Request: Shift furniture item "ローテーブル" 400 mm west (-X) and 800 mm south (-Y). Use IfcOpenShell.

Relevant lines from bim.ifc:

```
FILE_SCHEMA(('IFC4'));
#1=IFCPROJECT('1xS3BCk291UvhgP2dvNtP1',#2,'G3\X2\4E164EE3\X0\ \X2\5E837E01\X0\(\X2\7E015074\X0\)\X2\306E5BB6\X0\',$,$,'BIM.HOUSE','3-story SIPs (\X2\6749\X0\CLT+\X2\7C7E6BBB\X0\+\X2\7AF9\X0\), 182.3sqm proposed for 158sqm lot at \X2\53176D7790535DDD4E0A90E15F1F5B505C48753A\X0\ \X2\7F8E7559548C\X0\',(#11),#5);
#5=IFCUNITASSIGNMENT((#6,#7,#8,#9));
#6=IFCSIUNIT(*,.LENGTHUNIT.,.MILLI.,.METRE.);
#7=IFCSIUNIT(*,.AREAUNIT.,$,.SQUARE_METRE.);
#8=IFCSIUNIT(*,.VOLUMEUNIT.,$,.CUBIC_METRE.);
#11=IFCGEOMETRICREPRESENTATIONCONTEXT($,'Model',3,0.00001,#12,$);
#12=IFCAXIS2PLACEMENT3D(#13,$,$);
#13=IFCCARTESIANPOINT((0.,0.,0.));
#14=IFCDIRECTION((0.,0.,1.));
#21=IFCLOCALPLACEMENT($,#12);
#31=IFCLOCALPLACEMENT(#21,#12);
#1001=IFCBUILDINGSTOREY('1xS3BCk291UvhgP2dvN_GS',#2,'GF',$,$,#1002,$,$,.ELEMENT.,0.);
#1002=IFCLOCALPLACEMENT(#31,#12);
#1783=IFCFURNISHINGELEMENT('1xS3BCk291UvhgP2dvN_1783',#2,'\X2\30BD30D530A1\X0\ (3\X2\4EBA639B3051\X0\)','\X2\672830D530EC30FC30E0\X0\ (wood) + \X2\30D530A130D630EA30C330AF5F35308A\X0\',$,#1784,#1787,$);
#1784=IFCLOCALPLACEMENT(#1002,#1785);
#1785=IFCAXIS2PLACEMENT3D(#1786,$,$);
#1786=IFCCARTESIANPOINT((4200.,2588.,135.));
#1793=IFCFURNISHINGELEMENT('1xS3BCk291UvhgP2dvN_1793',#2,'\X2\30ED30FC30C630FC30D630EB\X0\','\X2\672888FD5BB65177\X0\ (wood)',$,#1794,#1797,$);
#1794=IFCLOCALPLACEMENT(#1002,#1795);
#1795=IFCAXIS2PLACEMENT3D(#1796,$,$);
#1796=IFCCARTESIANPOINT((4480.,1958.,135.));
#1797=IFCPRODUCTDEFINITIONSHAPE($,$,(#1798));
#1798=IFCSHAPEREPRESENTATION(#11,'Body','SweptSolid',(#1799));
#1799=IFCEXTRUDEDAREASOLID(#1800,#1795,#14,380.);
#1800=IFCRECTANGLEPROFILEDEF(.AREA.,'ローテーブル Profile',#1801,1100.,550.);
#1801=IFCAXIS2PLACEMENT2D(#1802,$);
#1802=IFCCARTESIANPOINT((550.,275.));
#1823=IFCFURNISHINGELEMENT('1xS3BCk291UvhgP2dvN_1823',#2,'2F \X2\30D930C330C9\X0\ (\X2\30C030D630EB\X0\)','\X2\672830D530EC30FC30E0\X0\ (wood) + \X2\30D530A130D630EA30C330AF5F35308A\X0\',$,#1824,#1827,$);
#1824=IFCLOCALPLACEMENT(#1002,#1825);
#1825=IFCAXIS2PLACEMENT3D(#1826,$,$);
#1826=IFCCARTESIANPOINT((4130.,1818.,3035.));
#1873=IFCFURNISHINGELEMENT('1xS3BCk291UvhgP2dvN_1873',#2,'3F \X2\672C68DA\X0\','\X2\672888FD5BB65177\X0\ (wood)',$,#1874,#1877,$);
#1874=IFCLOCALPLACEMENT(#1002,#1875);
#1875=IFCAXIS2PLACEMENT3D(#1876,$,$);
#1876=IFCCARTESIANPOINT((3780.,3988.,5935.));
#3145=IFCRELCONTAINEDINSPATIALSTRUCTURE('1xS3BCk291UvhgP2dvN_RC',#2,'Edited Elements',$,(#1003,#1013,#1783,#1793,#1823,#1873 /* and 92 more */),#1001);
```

```python
import ifcopenshell
import ifcopenshell.api.geometry
import ifcopenshell.util.placement
import ifcopenshell.util.unit

model = ifcopenshell.open("bim.ifc")
unit_scale = ifcopenshell.util.unit.calculate_unit_scale(model)

item = model.by_guid("1xS3BCk291UvhgP2dvN_1793")
matrix = ifcopenshell.util.placement.get_local_placement(item.ObjectPlacement)
matrix[0, 3] -= 0.4 / unit_scale
matrix[1, 3] -= 0.8 / unit_scale
ifcopenshell.api.geometry.edit_object_placement(model, product=item, matrix=matrix, is_si=False)

print(ifcopenshell.util.placement.get_local_placement(item.ObjectPlacement).round(3) + 0.0)

model.write("bim-out.ifc")
```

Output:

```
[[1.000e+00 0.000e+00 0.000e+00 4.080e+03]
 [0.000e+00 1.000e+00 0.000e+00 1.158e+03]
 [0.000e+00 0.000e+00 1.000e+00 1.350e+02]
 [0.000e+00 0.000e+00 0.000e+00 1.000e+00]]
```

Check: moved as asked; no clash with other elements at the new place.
